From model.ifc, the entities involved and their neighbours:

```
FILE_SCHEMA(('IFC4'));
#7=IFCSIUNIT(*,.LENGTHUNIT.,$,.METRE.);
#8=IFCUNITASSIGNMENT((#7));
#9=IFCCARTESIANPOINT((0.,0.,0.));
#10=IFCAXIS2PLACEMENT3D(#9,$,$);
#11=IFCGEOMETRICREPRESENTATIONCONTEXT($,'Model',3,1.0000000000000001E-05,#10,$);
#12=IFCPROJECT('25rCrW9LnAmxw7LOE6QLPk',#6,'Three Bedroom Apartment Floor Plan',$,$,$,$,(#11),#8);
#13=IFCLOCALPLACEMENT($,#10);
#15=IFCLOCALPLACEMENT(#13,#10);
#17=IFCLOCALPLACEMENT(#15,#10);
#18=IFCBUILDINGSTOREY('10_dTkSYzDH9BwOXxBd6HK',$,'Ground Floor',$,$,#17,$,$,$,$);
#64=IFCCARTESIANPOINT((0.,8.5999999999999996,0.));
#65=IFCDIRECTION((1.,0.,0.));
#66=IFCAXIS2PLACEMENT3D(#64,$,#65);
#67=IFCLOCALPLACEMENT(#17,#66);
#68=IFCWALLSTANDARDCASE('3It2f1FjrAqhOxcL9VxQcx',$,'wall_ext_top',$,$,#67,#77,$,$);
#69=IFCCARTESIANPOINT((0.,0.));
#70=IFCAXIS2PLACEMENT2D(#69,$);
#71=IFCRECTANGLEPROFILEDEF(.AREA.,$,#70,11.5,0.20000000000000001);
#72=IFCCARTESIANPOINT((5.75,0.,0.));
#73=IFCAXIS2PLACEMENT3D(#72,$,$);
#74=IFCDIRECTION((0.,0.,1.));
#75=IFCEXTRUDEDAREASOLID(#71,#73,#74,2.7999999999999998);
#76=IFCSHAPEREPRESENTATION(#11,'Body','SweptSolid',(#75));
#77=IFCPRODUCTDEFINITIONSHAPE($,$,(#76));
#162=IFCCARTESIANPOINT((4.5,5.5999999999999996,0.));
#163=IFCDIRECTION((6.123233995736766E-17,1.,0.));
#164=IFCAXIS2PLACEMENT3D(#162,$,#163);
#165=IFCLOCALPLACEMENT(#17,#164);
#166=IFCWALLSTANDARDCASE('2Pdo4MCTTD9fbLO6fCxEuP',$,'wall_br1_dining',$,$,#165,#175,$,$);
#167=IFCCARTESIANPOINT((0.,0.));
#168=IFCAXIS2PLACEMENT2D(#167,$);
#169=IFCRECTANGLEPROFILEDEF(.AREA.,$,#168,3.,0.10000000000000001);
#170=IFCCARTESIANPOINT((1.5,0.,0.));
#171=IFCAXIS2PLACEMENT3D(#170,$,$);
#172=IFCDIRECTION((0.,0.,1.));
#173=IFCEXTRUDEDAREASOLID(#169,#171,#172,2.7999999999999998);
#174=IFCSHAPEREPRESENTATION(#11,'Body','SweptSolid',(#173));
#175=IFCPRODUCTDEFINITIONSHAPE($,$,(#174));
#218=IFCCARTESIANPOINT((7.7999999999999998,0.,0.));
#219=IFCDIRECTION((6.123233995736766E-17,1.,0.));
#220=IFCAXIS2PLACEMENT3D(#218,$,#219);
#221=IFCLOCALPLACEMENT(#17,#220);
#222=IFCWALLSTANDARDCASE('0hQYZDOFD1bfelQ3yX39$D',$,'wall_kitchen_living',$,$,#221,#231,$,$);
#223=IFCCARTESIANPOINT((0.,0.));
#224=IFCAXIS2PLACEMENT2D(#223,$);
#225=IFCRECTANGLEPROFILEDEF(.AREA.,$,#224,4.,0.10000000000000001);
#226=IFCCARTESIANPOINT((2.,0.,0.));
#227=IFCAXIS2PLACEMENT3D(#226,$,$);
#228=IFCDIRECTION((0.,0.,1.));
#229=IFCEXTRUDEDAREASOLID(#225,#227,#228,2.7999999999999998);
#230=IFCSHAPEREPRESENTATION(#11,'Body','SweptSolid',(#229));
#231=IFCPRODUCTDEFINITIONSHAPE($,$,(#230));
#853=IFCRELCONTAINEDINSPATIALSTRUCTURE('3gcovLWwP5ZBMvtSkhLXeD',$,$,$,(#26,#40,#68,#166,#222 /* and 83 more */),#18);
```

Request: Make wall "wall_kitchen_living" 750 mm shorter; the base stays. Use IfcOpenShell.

```python
import ifcopenshell
import ifcopenshell.geom
import ifcopenshell.util.shape
import ifcopenshell.util.unit

model = ifcopenshell.open("model.ifc")
unit_scale = ifcopenshell.util.unit.calculate_unit_scale(model)
settings = ifcopenshell.geom.settings()


def volume(element):
    """Net volume in cubic metres, openings subtracted."""
    shape = ifcopenshell.geom.create_shape(settings, element)
    return ifcopenshell.util.shape.get_volume(shape.geometry)


wall = model.by_guid("0hQYZDOFD1bfelQ3yX39$D")
before = volume(wall)

body = next(r for r in wall.Representation.Representations if r.RepresentationIdentifier == "Body")
solid = body.Items[0]
old_height = solid.Depth
solid.Depth -= 0.75 / unit_scale
after = volume(wall)

print(f"height {old_height:g} -> {solid.Depth:g}, volume {before:.3f} -> {after:.3f} m3")

model.write("model-out.ifc")
```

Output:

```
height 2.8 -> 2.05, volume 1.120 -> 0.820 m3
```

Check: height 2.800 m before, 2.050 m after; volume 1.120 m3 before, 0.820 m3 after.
